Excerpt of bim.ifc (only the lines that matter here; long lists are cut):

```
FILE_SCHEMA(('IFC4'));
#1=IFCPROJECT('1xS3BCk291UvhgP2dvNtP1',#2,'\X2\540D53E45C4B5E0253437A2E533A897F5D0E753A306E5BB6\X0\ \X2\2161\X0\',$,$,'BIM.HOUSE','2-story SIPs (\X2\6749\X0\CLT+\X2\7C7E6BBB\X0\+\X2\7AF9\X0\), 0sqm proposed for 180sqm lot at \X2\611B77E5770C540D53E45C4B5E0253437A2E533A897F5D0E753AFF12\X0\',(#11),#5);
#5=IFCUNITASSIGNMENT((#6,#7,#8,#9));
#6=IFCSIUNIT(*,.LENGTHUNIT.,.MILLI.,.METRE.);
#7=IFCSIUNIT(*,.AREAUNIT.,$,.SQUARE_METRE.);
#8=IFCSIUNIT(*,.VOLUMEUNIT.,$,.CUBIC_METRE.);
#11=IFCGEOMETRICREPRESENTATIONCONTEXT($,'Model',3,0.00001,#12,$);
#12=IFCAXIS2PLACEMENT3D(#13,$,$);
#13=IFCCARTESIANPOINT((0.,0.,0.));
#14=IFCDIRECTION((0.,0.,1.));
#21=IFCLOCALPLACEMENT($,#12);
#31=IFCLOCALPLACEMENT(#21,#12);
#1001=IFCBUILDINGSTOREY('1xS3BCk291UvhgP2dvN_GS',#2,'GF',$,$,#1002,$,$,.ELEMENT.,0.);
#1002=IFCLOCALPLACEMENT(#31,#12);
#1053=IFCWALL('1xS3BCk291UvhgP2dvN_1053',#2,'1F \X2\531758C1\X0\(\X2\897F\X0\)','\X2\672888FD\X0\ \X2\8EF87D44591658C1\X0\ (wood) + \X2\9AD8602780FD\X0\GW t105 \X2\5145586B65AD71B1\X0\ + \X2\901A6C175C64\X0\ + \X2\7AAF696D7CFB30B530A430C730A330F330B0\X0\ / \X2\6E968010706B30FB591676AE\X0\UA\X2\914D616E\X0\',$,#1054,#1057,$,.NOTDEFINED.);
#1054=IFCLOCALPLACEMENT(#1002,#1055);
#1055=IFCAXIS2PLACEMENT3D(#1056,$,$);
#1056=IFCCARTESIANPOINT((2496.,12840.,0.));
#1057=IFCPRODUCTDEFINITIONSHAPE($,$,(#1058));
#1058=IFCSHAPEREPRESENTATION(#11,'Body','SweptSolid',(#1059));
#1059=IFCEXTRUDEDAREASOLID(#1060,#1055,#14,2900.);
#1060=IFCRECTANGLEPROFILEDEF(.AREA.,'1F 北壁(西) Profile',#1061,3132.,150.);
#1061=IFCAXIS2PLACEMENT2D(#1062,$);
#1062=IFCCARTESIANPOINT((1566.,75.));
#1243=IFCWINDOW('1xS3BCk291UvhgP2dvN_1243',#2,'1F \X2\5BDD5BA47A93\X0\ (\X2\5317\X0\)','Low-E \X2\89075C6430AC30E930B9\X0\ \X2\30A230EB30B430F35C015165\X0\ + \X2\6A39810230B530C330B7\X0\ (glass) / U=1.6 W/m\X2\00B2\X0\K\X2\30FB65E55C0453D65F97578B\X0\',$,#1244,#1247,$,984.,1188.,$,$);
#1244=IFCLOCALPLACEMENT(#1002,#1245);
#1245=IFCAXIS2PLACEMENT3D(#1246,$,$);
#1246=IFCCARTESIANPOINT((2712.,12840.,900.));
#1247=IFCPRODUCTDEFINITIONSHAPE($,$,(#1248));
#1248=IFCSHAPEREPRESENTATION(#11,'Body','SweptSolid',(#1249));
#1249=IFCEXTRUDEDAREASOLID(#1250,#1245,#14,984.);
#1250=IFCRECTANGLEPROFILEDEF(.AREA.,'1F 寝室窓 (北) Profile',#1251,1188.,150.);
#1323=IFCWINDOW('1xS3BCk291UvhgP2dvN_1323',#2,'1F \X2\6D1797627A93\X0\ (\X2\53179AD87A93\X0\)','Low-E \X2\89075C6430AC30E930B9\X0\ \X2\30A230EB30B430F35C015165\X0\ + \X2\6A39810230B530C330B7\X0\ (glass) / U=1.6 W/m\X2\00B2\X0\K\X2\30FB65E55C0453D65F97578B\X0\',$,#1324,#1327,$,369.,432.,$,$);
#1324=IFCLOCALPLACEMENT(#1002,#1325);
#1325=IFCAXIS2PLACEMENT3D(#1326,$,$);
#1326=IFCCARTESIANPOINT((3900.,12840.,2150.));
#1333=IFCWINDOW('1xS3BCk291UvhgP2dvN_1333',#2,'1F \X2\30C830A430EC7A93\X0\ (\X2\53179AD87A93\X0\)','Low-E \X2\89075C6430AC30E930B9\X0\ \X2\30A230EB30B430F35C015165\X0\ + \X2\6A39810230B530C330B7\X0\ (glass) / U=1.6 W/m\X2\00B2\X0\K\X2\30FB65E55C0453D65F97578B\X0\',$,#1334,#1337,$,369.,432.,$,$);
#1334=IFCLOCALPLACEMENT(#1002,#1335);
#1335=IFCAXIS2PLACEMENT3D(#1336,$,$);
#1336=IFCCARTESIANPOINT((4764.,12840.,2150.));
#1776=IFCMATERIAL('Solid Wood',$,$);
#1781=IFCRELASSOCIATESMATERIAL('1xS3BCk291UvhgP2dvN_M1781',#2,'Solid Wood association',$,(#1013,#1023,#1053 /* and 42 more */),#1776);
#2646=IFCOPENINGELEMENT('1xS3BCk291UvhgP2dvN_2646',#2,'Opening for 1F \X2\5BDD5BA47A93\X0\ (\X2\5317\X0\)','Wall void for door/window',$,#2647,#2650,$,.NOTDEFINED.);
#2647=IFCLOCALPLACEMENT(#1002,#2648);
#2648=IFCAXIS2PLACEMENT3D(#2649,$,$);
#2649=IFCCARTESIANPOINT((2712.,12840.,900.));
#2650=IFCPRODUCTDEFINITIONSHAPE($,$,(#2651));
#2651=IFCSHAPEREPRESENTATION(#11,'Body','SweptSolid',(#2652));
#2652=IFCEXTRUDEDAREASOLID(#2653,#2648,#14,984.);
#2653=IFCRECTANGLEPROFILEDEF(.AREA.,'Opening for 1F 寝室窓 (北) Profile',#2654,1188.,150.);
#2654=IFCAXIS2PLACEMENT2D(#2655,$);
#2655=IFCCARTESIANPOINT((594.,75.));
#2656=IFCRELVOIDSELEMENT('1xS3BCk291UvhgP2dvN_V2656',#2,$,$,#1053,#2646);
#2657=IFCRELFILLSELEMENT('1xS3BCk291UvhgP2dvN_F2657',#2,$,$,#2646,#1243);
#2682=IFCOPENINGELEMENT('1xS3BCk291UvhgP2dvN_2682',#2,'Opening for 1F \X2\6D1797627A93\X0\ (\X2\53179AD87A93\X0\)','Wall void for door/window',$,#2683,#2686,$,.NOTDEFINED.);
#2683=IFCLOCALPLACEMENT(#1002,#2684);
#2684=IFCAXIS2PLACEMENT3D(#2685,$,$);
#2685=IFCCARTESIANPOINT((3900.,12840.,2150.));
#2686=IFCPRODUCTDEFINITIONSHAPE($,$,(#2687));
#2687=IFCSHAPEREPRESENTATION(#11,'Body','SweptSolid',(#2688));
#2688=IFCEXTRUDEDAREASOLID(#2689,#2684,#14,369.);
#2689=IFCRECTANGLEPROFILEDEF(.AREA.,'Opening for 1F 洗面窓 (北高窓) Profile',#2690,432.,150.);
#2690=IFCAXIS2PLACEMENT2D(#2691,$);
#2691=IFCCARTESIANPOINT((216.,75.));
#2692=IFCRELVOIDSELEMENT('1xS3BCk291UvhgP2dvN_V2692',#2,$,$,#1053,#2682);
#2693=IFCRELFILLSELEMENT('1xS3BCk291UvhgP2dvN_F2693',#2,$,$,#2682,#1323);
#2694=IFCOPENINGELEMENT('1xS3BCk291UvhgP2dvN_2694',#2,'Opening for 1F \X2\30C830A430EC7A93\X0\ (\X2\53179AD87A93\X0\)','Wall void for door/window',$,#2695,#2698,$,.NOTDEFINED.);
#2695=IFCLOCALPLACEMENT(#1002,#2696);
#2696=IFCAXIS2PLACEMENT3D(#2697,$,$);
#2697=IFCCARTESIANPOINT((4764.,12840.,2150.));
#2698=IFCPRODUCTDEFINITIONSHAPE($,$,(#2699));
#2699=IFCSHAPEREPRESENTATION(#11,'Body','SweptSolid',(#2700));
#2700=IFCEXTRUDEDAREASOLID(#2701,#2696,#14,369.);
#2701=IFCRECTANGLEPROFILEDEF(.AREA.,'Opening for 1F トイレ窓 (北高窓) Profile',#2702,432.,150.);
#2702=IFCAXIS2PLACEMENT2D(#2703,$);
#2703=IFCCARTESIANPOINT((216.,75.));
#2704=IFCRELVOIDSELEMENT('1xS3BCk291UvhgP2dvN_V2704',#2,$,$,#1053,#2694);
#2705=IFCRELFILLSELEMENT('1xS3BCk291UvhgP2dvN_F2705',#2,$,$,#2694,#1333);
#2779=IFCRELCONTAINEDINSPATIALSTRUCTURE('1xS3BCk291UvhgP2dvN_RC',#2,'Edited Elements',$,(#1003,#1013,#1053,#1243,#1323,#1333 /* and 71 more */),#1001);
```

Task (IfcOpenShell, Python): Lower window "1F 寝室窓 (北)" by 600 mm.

```python
import numpy as np
import ifcopenshell
import ifcopenshell.api.geometry
import ifcopenshell.util.placement
import ifcopenshell.util.unit

model = ifcopenshell.open("bim.ifc")
unit_scale = ifcopenshell.util.unit.calculate_unit_scale(model)

window = model.by_guid("1xS3BCk291UvhgP2dvN_1243")
opening = window.FillsVoids[0].RelatingOpeningElement
dz = -600.0

shift = np.array([0.0, 0.0, dz])
# The window is not placed relative to its opening, so move both.
for product in (opening, window):
    matrix = ifcopenshell.util.placement.get_local_placement(product.ObjectPlacement)
    matrix[:3, 3] += shift
    ifcopenshell.api.geometry.edit_object_placement(model, product=product, matrix=matrix, is_si=False)

print(f"moved by {dz * unit_scale:+.3f} m")

model.write("bim_v2.ifc")
```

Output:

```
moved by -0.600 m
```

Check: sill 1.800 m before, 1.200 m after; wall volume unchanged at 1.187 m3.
